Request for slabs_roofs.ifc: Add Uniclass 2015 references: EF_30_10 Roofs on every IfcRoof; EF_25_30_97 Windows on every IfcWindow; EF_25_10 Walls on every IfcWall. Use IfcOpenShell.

First a look at what the model holds.

```python
import ifcopenshell

model = ifcopenshell.open("slabs_roofs.ifc")
print(model.schema)
print("classifications:", [c.Name for c in model.by_type("IfcClassification")])
for ifc_class in ("IfcDoor", "IfcRoof", "IfcStair", "IfcWall", "IfcWindow"):
    print(ifc_class, len(model.by_type(ifc_class)))
```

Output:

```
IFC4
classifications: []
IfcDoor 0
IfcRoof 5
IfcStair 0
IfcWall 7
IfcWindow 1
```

```python
import ifcopenshell
import ifcopenshell.api.classification

model = ifcopenshell.open("slabs_roofs.ifc")

system = ifcopenshell.api.classification.add_classification(model, classification="Uniclass 2015")

codes = {
    "IfcRoof": ("EF_30_10", "Roofs"),
    "IfcWindow": ("EF_25_30_97", "Windows"),
    "IfcWall": ("EF_25_10", "Walls"),
}
for ifc_class, (code, name) in codes.items():
    products = model.by_type(ifc_class)
    ifcopenshell.api.classification.add_reference(
        model, products=products, classification=system, identification=code, name=name
    )
    print(code, len(products))

model.write("slabs_roofs_v2.ifc")
```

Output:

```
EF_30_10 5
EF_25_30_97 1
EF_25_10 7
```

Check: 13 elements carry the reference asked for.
